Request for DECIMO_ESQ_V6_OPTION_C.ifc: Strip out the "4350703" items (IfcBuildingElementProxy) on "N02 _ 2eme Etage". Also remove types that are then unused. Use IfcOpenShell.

First a look at what the model holds.

```python
import ifcopenshell
import ifcopenshell.util.element

model = ifcopenshell.open("DECIMO_ESQ_V6_OPTION_C.ifc")
print(model.schema)
storey = next(s for s in model.by_type("IfcBuildingStorey") if s.Name == "N02 _ 2eme Etage")
proxies = [e for e in ifcopenshell.util.element.get_decomposition(storey) if e.is_a("IfcBuildingElementProxy")]
seen = {}
for e in proxies:
    element_type = ifcopenshell.util.element.get_type(e)
    name = element_type.Name if element_type not in (None, e) else None
    seen[name] = seen.get(name, 0) + 1
for name, count in sorted(seen.items(), key=str):
    print(count, "x", name)
```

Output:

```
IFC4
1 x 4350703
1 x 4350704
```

```python
import ifcopenshell
import ifcopenshell.api.root
import ifcopenshell.util.element

model = ifcopenshell.open("DECIMO_ESQ_V6_OPTION_C.ifc")

storey = next(s for s in model.by_type("IfcBuildingStorey") if s.Name == "N02 _ 2eme Etage")
proxies = [e for e in ifcopenshell.util.element.get_decomposition(storey) if e.is_a("IfcBuildingElementProxy")]
targets = [e for e in proxies if (t := ifcopenshell.util.element.get_type(e)) not in (None, e) and t.Name == "4350703"]
types = {ifcopenshell.util.element.get_type(e) for e in targets} - {None, *targets}

for e in targets:
    ifcopenshell.api.root.remove_product(model, product=e)
print(len(targets), "removed")

unused = [t for t in types if not ifcopenshell.util.element.get_types(t)]
for t in unused:
    ifcopenshell.api.root.remove_product(model, product=t)
print(len(unused), "unused types removed")

model.write("DECIMO_ESQ_V6_OPTION_C_edited.ifc")
```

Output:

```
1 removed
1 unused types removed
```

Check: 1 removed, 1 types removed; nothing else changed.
